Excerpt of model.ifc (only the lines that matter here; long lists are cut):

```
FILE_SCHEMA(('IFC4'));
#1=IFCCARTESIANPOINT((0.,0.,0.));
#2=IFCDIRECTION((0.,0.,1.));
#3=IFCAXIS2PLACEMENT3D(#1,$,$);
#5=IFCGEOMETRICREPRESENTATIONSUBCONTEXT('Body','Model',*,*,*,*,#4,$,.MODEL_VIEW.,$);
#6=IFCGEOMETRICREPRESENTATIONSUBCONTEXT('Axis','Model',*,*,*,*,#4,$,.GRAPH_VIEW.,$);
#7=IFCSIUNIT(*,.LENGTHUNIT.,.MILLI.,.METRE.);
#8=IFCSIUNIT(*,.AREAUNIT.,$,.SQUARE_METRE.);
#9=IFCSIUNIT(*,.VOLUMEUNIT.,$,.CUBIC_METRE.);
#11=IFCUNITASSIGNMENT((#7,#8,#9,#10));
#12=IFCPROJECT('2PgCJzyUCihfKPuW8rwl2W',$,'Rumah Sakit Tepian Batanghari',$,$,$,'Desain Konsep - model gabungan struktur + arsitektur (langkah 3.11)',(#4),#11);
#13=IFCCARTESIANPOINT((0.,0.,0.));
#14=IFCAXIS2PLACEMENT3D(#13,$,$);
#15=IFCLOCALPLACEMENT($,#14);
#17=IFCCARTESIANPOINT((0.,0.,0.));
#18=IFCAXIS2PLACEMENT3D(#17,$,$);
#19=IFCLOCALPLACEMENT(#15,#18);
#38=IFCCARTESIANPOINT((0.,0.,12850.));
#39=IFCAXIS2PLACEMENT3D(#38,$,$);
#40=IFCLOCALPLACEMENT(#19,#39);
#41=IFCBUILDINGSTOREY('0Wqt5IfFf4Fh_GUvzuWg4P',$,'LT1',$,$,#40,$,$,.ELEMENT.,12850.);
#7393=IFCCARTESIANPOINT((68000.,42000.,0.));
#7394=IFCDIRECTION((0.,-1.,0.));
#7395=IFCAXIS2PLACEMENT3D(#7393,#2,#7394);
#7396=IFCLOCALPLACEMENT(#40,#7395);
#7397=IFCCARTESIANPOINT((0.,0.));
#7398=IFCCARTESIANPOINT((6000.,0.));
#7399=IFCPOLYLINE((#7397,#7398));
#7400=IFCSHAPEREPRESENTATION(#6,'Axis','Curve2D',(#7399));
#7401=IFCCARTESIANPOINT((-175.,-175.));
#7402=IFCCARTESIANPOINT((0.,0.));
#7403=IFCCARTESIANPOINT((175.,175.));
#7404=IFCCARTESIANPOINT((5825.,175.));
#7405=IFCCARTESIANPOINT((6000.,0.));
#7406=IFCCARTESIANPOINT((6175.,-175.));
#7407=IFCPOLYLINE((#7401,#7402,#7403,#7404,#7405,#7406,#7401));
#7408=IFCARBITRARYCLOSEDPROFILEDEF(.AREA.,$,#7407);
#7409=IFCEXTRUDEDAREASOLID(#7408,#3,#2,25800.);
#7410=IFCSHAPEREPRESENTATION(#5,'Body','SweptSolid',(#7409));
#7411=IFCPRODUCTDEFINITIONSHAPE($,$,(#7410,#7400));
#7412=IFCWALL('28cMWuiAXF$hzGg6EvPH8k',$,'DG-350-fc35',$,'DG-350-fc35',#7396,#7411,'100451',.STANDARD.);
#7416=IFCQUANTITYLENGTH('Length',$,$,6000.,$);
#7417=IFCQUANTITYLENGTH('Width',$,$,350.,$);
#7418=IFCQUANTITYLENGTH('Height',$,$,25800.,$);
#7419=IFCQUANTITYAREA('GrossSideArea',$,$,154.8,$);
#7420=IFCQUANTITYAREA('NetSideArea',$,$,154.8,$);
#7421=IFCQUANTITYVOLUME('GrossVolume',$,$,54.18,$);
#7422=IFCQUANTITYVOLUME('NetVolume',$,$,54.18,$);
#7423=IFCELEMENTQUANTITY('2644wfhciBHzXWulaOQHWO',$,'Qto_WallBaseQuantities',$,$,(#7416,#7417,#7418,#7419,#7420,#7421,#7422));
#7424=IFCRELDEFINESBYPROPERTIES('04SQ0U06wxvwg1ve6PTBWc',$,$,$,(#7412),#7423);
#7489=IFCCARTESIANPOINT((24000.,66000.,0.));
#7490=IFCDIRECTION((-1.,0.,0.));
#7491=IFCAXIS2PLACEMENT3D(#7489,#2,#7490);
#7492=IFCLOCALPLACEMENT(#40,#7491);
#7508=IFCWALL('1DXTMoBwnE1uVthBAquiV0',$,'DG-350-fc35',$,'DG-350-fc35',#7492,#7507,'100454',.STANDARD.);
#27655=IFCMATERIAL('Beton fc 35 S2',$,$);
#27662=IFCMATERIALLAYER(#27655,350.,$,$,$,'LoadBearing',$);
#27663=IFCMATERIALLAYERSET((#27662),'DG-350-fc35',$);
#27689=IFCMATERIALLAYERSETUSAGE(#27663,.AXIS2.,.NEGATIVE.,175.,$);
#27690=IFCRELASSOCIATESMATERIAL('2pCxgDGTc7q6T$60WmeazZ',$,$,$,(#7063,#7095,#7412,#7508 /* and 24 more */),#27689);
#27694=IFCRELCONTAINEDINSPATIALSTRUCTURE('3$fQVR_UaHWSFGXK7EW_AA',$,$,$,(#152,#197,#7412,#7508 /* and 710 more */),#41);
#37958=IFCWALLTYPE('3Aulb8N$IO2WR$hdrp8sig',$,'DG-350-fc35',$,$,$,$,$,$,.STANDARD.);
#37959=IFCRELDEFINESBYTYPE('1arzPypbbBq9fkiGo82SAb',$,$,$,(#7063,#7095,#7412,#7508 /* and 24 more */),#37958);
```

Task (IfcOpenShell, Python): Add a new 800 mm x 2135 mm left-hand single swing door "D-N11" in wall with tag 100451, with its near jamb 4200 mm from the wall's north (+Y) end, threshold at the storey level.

```python
import numpy as np
import ifcopenshell
import ifcopenshell.api.feature
import ifcopenshell.api.geometry
import ifcopenshell.api.pset
import ifcopenshell.api.root
import ifcopenshell.api.spatial
import ifcopenshell.geom
import ifcopenshell.util.element
import ifcopenshell.util.placement
import ifcopenshell.util.representation
import ifcopenshell.util.shape
import ifcopenshell.util.unit

model = ifcopenshell.open("model.ifc")
unit_scale = ifcopenshell.util.unit.calculate_unit_scale(model)
area_scale = ifcopenshell.util.unit.calculate_unit_scale(model, "AREAUNIT")
volume_scale = ifcopenshell.util.unit.calculate_unit_scale(model, "VOLUMEUNIT")
settings = ifcopenshell.geom.settings()


def volume(element):
    """Net volume in cubic metres, openings subtracted."""
    shape = ifcopenshell.geom.create_shape(settings, element)
    return ifcopenshell.util.shape.get_volume(shape.geometry)


wall = model.by_id(7412)
storey = ifcopenshell.util.element.get_container(wall, ifc_class="IfcBuildingStorey")
context = ifcopenshell.util.representation.get_context(model, "Model", "Body", "MODEL_VIEW")
before = volume(wall)

width, height, from_end, sill = 0.8, 2.135, 4.2, 0.0  # metres

# The wall runs along its own X axis, and the end named is its -X end.
wall_shape = ifcopenshell.geom.create_shape(settings, wall)
x, y, z = ifcopenshell.util.shape.get_vertices(wall_shape.geometry).T
start = x.min() + from_end
face, thickness = float(y.min()), float(y.max() - y.min())
wall_matrix = ifcopenshell.util.placement.get_local_placement(wall.ObjectPlacement)
level = ifcopenshell.util.placement.get_local_placement(storey.ObjectPlacement)[2, 3]


def in_wall(x, y):
    """Placement at x, y metres in the wall's axes, at sill height."""
    matrix = wall_matrix.copy()
    matrix[:, 3] = wall_matrix @ np.array([x / unit_scale, y / unit_scale, 0.0, 1.0])
    matrix[2, 3] = level + sill / unit_scale
    return matrix


# Opening: a box that overshoots both wall faces by 50 mm.
opening = ifcopenshell.api.root.create_entity(model, ifc_class="IfcOpeningElement", predefined_type="OPENING")
box = ifcopenshell.api.geometry.add_wall_representation(
    model, context=context, length=width, height=height, thickness=thickness + 0.1
)
ifcopenshell.api.geometry.assign_representation(model, product=opening, representation=box)
ifcopenshell.api.geometry.edit_object_placement(model, product=opening, matrix=in_wall(start, face - 0.05), is_si=False)
ifcopenshell.api.feature.add_feature(model, feature=opening, element=wall)

door = ifcopenshell.api.root.create_entity(model, ifc_class="IfcDoor", name="D-N11", predefined_type="DOOR")
door.OverallWidth, door.OverallHeight = width / unit_scale, height / unit_scale
door.OperationType = "SINGLE_SWING_LEFT"
body = ifcopenshell.api.geometry.add_door_representation(
    model,
    context=context,
    overall_width=door.OverallWidth,
    overall_height=door.OverallHeight,
    operation_type="SINGLE_SWING_LEFT",
    lining_properties={"LiningDepth": thickness / unit_scale, "ThresholdDepth": thickness / unit_scale},
)
ifcopenshell.api.geometry.assign_representation(model, product=door, representation=body)
ifcopenshell.api.spatial.assign_container(model, products=[door], relating_structure=storey)
ifcopenshell.api.feature.add_filling(model, opening=opening, element=door)

# The lining spans the wall, so the door starts at the wall face.
ifcopenshell.api.geometry.edit_object_placement(model, product=door, matrix=in_wall(start, face), is_si=False)

after = volume(wall)

# Update the wall's stored quantities.
qto = model.by_id(ifcopenshell.util.element.get_pset(wall, "Qto_WallBaseQuantities", should_inherit=False)["id"])
ifcopenshell.api.pset.edit_qto(model, qto=qto, properties={
    "NetSideArea": after / thickness / area_scale,
    "NetVolume": after / volume_scale,
})

print(f"wall volume {before:.3f} -> {after:.3f} m3")

model.write("model_updated.ifc")
```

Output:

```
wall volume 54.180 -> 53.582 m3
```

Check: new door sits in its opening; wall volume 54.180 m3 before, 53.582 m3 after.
